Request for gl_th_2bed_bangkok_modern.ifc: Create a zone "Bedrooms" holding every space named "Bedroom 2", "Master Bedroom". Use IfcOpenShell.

First a look at what the model holds.

```python
import ifcopenshell

model = ifcopenshell.open("gl_th_2bed_bangkok_modern.ifc")
print(model.schema)
seen = {}
for space in model.by_type("IfcSpace"):
    seen[space.LongName] = seen.get(space.LongName, 0) + 1
for name, count in sorted(seen.items(), key=str):
    print(count, "x", name)
print("zones:", [z.Name for z in model.by_type("IfcZone")][:20])
```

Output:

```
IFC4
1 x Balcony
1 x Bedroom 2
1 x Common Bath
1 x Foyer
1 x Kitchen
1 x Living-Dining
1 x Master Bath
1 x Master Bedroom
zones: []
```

```python
import ifcopenshell
import ifcopenshell.api.group
import ifcopenshell.api.root

model = ifcopenshell.open("gl_th_2bed_bangkok_modern.ifc")

names = {"Bedroom 2", "Master Bedroom"}
spaces = [s for s in model.by_type("IfcSpace") if s.LongName in names]

zone = ifcopenshell.api.root.create_entity(model, ifc_class="IfcZone", name="Bedrooms")
ifcopenshell.api.group.assign_group(model, products=spaces, group=zone)
print(len(spaces), "spaces in", zone.Name)

model.write("gl_th_2bed_bangkok_modern_v2.ifc")
```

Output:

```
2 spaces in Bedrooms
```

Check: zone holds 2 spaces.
